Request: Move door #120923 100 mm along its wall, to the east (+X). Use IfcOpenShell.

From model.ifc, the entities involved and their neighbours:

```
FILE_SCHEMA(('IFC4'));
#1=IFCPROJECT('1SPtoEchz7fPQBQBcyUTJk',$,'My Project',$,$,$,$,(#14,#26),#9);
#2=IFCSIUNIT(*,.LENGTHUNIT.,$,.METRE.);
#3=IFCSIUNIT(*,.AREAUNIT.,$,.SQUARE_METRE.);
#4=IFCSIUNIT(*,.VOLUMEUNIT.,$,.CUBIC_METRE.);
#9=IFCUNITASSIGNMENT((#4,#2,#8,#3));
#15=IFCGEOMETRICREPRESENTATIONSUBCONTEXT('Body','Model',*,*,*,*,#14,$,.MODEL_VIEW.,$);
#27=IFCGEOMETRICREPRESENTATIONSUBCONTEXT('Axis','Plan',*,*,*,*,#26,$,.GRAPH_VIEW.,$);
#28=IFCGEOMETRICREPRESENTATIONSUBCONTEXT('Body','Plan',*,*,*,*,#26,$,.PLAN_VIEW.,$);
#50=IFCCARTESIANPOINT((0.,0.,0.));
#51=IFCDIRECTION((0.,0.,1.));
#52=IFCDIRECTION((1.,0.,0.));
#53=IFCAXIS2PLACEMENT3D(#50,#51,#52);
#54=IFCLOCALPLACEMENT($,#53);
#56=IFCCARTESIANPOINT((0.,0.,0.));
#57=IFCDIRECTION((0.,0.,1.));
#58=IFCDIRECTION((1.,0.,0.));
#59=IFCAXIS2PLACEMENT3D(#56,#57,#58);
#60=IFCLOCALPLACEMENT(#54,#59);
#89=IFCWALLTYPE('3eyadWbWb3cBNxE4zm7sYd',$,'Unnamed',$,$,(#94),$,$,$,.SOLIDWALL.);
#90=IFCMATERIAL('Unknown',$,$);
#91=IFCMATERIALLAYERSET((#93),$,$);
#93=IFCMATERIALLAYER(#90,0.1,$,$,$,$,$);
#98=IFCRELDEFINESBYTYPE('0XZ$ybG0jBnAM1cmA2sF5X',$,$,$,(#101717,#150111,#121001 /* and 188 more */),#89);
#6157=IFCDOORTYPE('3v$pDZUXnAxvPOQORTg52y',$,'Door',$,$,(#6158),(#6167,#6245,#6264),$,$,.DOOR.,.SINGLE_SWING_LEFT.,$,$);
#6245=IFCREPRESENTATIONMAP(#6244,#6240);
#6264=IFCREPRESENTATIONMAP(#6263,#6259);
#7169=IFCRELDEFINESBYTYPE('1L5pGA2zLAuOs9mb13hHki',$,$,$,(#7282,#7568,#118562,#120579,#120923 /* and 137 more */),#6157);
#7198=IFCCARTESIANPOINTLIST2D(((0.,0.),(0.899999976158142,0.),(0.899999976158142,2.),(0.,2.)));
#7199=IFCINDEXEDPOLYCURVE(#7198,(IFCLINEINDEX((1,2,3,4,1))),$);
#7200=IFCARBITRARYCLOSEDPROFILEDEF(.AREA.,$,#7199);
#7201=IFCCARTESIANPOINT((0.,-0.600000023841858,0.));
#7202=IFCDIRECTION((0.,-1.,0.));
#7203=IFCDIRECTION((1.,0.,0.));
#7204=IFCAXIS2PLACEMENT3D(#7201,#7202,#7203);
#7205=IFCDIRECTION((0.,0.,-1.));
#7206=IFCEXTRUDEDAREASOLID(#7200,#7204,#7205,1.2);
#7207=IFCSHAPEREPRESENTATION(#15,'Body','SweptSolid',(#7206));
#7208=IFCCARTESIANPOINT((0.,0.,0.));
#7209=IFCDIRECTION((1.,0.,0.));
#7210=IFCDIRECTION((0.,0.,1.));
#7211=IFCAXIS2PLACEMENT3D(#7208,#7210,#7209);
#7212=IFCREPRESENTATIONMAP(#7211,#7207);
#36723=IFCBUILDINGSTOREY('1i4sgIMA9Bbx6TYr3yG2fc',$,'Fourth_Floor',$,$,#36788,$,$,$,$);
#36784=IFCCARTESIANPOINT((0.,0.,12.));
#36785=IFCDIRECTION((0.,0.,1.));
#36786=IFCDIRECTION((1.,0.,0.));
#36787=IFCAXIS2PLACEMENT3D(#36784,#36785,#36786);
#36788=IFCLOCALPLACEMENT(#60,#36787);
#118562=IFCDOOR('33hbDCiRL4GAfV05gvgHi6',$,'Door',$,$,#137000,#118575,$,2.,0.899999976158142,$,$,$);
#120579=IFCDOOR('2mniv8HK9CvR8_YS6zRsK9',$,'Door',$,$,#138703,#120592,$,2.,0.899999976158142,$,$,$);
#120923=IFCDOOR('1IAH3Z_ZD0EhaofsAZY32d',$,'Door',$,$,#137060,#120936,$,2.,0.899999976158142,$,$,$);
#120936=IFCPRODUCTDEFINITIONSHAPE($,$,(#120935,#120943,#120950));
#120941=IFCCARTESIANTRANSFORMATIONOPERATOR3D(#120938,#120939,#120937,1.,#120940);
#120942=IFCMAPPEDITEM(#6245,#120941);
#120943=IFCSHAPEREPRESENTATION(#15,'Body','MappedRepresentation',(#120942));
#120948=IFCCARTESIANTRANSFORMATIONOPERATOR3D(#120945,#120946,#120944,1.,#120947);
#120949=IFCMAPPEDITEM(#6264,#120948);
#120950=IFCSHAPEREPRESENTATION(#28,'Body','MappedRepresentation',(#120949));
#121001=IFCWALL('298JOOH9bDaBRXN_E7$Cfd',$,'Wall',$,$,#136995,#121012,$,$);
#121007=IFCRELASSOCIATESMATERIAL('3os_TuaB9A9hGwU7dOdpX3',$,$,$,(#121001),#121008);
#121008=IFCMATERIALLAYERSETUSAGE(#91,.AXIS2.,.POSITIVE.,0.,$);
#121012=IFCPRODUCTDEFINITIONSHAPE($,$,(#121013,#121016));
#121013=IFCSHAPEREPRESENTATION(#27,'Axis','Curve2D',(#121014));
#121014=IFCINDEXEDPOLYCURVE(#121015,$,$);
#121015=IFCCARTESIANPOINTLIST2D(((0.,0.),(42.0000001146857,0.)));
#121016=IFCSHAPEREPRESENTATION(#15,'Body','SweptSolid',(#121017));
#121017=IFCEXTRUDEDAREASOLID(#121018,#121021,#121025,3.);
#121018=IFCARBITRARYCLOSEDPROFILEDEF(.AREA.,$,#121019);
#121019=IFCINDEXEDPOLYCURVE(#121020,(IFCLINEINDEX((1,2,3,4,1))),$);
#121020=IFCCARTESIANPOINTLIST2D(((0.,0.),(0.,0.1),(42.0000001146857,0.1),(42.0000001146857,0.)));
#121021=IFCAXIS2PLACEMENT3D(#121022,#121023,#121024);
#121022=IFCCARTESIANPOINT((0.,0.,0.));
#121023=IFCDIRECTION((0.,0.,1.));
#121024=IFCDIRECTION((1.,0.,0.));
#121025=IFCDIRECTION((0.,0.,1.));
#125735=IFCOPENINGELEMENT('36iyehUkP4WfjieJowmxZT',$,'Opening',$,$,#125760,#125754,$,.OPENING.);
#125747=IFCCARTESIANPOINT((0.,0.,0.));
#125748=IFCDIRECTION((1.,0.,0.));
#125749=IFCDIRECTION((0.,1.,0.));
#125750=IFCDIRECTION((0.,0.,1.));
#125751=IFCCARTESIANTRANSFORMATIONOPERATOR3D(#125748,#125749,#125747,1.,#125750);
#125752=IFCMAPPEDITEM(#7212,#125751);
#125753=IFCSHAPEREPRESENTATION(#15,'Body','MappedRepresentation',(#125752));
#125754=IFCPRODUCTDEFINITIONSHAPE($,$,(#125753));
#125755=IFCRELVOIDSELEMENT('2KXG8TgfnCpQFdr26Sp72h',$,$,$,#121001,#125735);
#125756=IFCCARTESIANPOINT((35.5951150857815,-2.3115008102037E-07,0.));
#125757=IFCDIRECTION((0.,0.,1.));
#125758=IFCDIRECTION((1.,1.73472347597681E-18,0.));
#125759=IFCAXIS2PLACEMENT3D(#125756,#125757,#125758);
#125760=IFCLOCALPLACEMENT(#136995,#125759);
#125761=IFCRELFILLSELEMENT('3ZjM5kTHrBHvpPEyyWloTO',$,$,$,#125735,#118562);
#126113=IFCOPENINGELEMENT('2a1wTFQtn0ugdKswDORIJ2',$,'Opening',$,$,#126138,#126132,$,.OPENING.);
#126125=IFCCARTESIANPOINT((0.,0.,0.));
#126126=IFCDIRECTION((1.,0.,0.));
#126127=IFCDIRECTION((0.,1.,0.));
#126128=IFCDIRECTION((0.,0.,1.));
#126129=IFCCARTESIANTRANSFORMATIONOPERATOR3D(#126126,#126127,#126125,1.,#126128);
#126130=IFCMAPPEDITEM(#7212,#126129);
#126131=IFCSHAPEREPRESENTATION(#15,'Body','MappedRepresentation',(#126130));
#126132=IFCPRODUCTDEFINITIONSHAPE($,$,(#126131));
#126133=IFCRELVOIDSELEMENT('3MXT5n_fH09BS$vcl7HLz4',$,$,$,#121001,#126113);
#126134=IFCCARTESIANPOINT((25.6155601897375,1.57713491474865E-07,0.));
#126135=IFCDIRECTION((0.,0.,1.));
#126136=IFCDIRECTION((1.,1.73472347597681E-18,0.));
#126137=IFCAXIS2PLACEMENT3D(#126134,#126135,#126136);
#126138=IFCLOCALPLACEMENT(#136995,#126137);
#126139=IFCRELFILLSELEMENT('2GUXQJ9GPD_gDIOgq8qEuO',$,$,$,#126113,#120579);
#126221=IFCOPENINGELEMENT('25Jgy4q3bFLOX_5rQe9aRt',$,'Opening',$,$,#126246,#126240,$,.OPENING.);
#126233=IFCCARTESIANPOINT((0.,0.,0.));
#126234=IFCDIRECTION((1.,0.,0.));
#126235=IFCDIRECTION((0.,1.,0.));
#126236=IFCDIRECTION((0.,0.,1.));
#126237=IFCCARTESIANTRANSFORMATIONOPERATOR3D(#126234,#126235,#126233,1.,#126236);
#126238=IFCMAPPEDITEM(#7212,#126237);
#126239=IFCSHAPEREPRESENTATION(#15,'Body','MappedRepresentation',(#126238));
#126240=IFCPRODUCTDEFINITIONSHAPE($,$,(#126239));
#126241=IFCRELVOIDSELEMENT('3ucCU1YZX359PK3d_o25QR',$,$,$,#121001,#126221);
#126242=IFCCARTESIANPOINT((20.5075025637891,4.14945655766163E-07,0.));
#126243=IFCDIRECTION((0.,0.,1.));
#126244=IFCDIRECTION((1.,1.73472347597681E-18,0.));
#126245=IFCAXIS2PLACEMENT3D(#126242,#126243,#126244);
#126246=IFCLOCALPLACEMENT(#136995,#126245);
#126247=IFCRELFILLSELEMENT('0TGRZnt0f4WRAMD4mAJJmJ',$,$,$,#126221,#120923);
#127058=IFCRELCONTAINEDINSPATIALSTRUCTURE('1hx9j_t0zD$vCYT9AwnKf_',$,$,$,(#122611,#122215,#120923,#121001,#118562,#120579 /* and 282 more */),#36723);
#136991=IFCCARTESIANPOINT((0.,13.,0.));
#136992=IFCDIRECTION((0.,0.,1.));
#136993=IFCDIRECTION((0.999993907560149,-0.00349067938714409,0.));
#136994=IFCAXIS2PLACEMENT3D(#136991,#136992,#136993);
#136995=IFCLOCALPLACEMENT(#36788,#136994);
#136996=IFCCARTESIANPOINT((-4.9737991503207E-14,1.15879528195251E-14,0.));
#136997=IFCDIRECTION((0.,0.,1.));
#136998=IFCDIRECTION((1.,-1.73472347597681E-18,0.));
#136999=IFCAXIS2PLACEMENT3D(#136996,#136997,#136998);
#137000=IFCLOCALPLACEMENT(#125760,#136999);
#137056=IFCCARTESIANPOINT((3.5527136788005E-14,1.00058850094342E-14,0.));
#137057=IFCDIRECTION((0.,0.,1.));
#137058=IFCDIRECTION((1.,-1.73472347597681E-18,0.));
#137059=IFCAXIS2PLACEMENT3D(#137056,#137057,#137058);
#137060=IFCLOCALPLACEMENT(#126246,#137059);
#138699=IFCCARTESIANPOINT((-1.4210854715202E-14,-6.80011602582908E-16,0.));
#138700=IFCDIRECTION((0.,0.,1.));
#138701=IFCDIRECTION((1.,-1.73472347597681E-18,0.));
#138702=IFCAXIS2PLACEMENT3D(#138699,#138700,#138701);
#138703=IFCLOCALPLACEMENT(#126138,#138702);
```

```python
import ifcopenshell
import ifcopenshell.api.geometry
import ifcopenshell.util.placement
import ifcopenshell.util.unit

model = ifcopenshell.open("model.ifc")
unit_scale = ifcopenshell.util.unit.calculate_unit_scale(model)

door = model.by_guid("1IAH3Z_ZD0EhaofsAZY32d")
opening = door.FillsVoids[0].RelatingOpeningElement
wall = opening.VoidsElements[0].RelatingBuildingElement

wall_matrix = ifcopenshell.util.placement.get_local_placement(wall.ObjectPlacement)
shift = wall_matrix[:3, 0] * 0.1 / unit_scale
before = ifcopenshell.util.placement.get_local_placement(door.ObjectPlacement)[:3, 3].copy()

# The door is placed relative to its opening, so it follows when the opening moves.
matrix = ifcopenshell.util.placement.get_local_placement(opening.ObjectPlacement)
matrix[:3, 3] += shift
ifcopenshell.api.geometry.edit_object_placement(
    model, product=opening, matrix=matrix, is_si=False, should_transform_children=True
)

after = ifcopenshell.util.placement.get_local_placement(door.ObjectPlacement)[:3, 3]
print("door moved by", (after - before).round(3) + 0.0)

model.write("model-out.ifc")
```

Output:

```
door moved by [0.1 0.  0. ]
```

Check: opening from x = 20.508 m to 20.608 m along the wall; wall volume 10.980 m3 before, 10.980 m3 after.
